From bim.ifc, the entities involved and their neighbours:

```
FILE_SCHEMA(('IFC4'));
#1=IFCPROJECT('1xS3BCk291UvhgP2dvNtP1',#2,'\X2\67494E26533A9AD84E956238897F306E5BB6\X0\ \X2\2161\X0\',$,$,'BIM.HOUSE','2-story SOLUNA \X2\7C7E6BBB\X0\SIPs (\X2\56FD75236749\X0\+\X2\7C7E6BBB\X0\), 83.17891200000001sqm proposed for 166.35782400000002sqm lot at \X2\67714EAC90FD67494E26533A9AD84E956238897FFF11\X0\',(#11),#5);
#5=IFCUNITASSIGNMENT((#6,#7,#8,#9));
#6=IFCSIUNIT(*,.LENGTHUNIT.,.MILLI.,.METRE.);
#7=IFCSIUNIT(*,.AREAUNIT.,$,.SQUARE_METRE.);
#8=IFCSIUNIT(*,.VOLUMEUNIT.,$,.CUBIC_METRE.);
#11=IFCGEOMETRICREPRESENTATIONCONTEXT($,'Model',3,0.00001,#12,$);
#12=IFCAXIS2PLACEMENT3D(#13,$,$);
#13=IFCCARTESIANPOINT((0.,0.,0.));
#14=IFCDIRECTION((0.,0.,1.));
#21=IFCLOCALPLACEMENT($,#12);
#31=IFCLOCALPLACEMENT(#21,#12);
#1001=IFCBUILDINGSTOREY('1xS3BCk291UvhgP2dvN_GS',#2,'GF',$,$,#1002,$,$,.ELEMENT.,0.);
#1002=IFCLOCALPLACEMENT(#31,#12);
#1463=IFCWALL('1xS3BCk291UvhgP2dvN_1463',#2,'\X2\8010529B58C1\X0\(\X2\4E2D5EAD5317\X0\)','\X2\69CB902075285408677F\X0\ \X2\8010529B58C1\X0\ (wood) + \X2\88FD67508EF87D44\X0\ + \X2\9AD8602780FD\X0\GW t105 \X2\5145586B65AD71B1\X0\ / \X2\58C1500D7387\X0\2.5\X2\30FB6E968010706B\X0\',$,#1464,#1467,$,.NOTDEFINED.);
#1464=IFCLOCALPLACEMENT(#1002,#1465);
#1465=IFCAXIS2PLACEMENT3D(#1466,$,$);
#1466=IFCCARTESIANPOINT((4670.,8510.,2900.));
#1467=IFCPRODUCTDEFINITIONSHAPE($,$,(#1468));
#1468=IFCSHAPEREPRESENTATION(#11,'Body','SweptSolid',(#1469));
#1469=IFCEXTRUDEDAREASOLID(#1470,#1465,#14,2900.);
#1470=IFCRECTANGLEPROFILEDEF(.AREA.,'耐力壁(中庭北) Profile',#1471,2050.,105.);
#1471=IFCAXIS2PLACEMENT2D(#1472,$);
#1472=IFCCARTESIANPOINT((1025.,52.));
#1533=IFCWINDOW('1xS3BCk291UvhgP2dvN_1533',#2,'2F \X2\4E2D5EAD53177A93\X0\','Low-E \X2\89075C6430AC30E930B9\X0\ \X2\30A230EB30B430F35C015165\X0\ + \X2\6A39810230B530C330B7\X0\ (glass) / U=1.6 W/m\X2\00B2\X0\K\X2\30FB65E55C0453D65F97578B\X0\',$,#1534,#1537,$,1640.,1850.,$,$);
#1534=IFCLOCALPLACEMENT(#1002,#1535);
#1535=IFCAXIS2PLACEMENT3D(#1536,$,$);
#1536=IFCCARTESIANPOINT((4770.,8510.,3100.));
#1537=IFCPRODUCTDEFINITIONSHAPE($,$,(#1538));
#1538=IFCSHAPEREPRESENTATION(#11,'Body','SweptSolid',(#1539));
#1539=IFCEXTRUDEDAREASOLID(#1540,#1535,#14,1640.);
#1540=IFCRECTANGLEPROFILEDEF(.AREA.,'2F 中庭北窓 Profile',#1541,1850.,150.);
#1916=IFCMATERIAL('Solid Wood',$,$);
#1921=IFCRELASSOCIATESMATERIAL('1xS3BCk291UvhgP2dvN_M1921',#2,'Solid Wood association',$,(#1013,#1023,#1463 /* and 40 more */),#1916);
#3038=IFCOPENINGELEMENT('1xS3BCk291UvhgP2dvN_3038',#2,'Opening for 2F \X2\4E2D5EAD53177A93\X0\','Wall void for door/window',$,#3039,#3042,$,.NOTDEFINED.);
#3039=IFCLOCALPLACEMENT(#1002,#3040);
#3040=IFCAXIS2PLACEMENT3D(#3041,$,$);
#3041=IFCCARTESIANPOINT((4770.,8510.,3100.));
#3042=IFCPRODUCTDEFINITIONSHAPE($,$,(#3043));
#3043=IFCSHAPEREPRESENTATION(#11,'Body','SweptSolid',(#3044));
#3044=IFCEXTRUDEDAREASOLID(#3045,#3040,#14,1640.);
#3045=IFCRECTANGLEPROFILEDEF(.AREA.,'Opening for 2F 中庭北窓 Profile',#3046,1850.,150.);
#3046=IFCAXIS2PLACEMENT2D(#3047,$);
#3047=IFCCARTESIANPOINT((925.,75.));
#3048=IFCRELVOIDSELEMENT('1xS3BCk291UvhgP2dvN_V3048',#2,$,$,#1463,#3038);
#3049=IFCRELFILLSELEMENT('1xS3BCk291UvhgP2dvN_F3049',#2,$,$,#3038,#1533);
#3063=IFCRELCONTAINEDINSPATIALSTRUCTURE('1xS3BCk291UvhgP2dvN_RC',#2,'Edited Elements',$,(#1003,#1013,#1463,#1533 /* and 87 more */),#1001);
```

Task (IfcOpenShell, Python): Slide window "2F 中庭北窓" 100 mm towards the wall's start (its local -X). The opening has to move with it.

```python
import ifcopenshell
import ifcopenshell.api.geometry
import ifcopenshell.util.placement

model = ifcopenshell.open("bim.ifc")

window = model.by_guid("1xS3BCk291UvhgP2dvN_1533")
opening = window.FillsVoids[0].RelatingOpeningElement
wall = opening.VoidsElements[0].RelatingBuildingElement

wall_matrix = ifcopenshell.util.placement.get_local_placement(wall.ObjectPlacement)
shift = wall_matrix[:3, 0] * -100.0
before = ifcopenshell.util.placement.get_local_placement(window.ObjectPlacement)[:3, 3].copy()

# The window is not placed relative to its opening, so move both.
for product in (opening, window):
    matrix = ifcopenshell.util.placement.get_local_placement(product.ObjectPlacement)
    matrix[:3, 3] += shift
    ifcopenshell.api.geometry.edit_object_placement(model, product=product, matrix=matrix, is_si=False)

after = ifcopenshell.util.placement.get_local_placement(window.ObjectPlacement)[:3, 3]
print("window moved by", (after - before).round(3) + 0.0)

model.write("bim_edited.ifc")
```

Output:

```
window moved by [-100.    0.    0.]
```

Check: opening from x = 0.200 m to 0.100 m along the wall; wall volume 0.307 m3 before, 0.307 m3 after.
